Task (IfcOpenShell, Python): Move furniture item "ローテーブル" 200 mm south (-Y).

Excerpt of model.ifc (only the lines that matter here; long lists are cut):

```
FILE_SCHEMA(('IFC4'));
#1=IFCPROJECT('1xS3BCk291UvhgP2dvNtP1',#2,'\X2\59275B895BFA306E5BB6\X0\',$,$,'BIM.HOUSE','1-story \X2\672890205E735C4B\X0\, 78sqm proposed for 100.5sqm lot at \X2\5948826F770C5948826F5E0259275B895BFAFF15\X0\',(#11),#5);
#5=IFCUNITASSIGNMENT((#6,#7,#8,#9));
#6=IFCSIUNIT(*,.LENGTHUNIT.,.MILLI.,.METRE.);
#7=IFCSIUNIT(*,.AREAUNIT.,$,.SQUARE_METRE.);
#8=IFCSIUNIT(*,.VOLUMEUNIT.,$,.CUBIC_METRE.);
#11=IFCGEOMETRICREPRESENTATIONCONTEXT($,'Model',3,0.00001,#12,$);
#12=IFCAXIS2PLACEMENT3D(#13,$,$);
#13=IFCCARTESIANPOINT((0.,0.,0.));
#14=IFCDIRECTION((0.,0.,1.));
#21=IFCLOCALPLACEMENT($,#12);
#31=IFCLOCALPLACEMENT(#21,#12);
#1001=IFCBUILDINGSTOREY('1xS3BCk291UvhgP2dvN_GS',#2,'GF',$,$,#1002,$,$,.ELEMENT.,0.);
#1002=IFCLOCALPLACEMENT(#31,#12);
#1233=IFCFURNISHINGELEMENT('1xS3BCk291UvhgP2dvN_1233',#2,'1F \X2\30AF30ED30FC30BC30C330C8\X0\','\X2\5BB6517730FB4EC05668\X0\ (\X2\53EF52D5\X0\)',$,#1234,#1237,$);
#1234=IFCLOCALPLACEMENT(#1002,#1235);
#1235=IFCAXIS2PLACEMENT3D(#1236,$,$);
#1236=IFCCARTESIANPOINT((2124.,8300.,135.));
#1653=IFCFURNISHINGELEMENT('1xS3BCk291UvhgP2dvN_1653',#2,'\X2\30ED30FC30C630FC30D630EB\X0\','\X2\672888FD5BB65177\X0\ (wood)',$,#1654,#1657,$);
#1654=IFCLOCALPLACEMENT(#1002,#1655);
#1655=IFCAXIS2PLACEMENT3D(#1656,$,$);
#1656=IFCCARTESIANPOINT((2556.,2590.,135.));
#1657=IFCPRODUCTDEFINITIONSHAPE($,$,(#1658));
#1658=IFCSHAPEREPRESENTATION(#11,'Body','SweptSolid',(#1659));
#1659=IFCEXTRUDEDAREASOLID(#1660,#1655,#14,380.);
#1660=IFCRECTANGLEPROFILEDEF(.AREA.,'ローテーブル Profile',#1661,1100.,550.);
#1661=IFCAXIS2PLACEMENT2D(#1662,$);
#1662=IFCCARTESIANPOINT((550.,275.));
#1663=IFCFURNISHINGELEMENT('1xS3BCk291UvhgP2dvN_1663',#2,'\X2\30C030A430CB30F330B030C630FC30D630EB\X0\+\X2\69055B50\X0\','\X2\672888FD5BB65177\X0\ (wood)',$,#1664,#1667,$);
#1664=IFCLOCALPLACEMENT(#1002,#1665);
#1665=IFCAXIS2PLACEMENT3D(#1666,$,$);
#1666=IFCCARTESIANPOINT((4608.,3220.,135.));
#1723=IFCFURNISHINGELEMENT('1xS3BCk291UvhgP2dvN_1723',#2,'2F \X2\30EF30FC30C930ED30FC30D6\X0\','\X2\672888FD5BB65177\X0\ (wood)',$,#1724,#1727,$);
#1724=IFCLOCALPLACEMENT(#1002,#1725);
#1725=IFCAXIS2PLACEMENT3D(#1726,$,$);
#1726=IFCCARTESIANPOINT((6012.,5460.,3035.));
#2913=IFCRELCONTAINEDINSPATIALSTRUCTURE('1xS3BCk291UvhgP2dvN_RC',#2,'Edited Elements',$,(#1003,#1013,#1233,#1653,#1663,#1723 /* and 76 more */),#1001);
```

```python
import ifcopenshell
import ifcopenshell.api.geometry
import ifcopenshell.util.placement
import ifcopenshell.util.unit

model = ifcopenshell.open("model.ifc")
unit_scale = ifcopenshell.util.unit.calculate_unit_scale(model)

item = model.by_guid("1xS3BCk291UvhgP2dvN_1653")
matrix = ifcopenshell.util.placement.get_local_placement(item.ObjectPlacement)
matrix[1, 3] -= 0.2 / unit_scale
ifcopenshell.api.geometry.edit_object_placement(model, product=item, matrix=matrix, is_si=False)

print(ifcopenshell.util.placement.get_local_placement(item.ObjectPlacement).round(3) + 0.0)

model.write("model_updated.ifc")
```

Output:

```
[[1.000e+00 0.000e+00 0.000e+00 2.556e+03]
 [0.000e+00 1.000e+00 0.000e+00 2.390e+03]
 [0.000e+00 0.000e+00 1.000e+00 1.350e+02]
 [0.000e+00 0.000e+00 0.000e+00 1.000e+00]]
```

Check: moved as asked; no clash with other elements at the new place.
